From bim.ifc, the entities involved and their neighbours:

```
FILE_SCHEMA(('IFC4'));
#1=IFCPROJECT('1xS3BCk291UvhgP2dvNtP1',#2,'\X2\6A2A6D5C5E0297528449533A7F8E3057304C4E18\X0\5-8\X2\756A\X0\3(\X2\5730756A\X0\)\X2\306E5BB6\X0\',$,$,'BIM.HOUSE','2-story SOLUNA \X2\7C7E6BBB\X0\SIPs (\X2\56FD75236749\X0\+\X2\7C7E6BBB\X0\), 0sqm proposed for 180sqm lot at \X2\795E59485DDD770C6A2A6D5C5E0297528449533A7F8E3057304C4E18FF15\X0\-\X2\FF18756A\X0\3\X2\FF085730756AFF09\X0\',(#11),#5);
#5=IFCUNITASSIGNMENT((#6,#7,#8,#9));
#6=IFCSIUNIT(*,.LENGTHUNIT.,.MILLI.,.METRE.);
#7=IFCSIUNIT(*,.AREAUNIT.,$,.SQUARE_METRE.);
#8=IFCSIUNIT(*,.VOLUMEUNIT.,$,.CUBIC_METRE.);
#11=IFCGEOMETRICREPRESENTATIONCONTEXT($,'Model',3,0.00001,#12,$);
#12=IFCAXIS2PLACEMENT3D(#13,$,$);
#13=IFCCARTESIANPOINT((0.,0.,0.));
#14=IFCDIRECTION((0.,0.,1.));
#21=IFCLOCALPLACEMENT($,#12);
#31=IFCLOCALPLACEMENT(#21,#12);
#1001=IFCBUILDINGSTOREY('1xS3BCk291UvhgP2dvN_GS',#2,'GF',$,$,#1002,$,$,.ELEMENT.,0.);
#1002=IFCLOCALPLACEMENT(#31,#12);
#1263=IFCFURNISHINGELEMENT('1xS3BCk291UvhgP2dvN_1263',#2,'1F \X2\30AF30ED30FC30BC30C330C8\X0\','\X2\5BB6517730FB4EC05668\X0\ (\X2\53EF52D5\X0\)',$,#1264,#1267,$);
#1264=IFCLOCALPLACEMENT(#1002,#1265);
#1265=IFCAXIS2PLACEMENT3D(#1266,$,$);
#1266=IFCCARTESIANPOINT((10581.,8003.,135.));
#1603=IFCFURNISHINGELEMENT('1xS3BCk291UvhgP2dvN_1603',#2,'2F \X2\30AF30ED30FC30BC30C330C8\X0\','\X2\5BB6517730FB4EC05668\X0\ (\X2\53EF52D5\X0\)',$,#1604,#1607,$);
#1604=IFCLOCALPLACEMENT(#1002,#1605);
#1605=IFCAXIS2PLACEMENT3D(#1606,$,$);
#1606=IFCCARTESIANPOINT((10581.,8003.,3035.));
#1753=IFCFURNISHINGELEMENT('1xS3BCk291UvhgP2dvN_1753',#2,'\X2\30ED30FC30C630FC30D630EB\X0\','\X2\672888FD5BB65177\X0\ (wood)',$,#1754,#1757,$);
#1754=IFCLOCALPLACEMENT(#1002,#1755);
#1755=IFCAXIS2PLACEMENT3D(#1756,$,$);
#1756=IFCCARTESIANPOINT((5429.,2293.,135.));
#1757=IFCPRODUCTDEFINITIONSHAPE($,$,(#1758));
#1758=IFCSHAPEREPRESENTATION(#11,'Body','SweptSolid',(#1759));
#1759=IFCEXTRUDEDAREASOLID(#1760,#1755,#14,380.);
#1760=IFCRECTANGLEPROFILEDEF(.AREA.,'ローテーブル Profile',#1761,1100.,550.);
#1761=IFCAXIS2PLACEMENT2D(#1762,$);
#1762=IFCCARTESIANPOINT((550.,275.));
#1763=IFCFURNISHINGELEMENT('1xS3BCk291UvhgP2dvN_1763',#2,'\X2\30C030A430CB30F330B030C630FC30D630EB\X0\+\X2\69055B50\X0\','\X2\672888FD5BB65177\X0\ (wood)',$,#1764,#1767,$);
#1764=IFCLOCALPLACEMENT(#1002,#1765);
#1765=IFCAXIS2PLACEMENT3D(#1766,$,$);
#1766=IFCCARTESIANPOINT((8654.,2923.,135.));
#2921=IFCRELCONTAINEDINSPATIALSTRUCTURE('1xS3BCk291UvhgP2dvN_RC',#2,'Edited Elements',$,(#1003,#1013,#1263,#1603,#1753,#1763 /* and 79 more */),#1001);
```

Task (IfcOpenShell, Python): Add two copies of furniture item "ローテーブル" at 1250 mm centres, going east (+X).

```python
import numpy as np
import ifcopenshell
import ifcopenshell.api.geometry
import ifcopenshell.api.root
import ifcopenshell.util.element
import ifcopenshell.util.placement
import ifcopenshell.util.unit

model = ifcopenshell.open("bim.ifc")
unit_scale = ifcopenshell.util.unit.calculate_unit_scale(model)


def reuse_history(source, copy):
    """copy_class also copies each property set's owner history, people and application; keep the originals."""
    for rel in copy.IsDefinedBy:
        if rel.is_a("IfcRelDefinesByProperties") and (history := rel.RelatingPropertyDefinition.OwnerHistory):
            rel.RelatingPropertyDefinition.OwnerHistory = source.OwnerHistory
            ifcopenshell.util.element.remove_deep2(model, history)


source = model.by_guid("1xS3BCk291UvhgP2dvN_1753")
base = ifcopenshell.util.placement.get_local_placement(source.ObjectPlacement)
step = np.array([1.0, 0.0, 0.0]) * 1.25 / unit_scale

for i in range(1, 3):
    copy = ifcopenshell.api.root.copy_class(model, product=source)
    copy.Representation = ifcopenshell.util.element.copy_deep(
        model, source.Representation, exclude=["IfcGeometricRepresentationContext", "IfcRepresentationMap"]
    )
    reuse_history(source, copy)
    matrix = base.copy()
    matrix[:3, 3] += i * step
    print("added at", matrix[:3, 3].round(3) + 0.0)
    ifcopenshell.api.geometry.edit_object_placement(model, product=copy, matrix=matrix, is_si=False)

model.write("bim_edited.ifc")
```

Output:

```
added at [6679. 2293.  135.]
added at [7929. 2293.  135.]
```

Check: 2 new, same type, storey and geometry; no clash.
